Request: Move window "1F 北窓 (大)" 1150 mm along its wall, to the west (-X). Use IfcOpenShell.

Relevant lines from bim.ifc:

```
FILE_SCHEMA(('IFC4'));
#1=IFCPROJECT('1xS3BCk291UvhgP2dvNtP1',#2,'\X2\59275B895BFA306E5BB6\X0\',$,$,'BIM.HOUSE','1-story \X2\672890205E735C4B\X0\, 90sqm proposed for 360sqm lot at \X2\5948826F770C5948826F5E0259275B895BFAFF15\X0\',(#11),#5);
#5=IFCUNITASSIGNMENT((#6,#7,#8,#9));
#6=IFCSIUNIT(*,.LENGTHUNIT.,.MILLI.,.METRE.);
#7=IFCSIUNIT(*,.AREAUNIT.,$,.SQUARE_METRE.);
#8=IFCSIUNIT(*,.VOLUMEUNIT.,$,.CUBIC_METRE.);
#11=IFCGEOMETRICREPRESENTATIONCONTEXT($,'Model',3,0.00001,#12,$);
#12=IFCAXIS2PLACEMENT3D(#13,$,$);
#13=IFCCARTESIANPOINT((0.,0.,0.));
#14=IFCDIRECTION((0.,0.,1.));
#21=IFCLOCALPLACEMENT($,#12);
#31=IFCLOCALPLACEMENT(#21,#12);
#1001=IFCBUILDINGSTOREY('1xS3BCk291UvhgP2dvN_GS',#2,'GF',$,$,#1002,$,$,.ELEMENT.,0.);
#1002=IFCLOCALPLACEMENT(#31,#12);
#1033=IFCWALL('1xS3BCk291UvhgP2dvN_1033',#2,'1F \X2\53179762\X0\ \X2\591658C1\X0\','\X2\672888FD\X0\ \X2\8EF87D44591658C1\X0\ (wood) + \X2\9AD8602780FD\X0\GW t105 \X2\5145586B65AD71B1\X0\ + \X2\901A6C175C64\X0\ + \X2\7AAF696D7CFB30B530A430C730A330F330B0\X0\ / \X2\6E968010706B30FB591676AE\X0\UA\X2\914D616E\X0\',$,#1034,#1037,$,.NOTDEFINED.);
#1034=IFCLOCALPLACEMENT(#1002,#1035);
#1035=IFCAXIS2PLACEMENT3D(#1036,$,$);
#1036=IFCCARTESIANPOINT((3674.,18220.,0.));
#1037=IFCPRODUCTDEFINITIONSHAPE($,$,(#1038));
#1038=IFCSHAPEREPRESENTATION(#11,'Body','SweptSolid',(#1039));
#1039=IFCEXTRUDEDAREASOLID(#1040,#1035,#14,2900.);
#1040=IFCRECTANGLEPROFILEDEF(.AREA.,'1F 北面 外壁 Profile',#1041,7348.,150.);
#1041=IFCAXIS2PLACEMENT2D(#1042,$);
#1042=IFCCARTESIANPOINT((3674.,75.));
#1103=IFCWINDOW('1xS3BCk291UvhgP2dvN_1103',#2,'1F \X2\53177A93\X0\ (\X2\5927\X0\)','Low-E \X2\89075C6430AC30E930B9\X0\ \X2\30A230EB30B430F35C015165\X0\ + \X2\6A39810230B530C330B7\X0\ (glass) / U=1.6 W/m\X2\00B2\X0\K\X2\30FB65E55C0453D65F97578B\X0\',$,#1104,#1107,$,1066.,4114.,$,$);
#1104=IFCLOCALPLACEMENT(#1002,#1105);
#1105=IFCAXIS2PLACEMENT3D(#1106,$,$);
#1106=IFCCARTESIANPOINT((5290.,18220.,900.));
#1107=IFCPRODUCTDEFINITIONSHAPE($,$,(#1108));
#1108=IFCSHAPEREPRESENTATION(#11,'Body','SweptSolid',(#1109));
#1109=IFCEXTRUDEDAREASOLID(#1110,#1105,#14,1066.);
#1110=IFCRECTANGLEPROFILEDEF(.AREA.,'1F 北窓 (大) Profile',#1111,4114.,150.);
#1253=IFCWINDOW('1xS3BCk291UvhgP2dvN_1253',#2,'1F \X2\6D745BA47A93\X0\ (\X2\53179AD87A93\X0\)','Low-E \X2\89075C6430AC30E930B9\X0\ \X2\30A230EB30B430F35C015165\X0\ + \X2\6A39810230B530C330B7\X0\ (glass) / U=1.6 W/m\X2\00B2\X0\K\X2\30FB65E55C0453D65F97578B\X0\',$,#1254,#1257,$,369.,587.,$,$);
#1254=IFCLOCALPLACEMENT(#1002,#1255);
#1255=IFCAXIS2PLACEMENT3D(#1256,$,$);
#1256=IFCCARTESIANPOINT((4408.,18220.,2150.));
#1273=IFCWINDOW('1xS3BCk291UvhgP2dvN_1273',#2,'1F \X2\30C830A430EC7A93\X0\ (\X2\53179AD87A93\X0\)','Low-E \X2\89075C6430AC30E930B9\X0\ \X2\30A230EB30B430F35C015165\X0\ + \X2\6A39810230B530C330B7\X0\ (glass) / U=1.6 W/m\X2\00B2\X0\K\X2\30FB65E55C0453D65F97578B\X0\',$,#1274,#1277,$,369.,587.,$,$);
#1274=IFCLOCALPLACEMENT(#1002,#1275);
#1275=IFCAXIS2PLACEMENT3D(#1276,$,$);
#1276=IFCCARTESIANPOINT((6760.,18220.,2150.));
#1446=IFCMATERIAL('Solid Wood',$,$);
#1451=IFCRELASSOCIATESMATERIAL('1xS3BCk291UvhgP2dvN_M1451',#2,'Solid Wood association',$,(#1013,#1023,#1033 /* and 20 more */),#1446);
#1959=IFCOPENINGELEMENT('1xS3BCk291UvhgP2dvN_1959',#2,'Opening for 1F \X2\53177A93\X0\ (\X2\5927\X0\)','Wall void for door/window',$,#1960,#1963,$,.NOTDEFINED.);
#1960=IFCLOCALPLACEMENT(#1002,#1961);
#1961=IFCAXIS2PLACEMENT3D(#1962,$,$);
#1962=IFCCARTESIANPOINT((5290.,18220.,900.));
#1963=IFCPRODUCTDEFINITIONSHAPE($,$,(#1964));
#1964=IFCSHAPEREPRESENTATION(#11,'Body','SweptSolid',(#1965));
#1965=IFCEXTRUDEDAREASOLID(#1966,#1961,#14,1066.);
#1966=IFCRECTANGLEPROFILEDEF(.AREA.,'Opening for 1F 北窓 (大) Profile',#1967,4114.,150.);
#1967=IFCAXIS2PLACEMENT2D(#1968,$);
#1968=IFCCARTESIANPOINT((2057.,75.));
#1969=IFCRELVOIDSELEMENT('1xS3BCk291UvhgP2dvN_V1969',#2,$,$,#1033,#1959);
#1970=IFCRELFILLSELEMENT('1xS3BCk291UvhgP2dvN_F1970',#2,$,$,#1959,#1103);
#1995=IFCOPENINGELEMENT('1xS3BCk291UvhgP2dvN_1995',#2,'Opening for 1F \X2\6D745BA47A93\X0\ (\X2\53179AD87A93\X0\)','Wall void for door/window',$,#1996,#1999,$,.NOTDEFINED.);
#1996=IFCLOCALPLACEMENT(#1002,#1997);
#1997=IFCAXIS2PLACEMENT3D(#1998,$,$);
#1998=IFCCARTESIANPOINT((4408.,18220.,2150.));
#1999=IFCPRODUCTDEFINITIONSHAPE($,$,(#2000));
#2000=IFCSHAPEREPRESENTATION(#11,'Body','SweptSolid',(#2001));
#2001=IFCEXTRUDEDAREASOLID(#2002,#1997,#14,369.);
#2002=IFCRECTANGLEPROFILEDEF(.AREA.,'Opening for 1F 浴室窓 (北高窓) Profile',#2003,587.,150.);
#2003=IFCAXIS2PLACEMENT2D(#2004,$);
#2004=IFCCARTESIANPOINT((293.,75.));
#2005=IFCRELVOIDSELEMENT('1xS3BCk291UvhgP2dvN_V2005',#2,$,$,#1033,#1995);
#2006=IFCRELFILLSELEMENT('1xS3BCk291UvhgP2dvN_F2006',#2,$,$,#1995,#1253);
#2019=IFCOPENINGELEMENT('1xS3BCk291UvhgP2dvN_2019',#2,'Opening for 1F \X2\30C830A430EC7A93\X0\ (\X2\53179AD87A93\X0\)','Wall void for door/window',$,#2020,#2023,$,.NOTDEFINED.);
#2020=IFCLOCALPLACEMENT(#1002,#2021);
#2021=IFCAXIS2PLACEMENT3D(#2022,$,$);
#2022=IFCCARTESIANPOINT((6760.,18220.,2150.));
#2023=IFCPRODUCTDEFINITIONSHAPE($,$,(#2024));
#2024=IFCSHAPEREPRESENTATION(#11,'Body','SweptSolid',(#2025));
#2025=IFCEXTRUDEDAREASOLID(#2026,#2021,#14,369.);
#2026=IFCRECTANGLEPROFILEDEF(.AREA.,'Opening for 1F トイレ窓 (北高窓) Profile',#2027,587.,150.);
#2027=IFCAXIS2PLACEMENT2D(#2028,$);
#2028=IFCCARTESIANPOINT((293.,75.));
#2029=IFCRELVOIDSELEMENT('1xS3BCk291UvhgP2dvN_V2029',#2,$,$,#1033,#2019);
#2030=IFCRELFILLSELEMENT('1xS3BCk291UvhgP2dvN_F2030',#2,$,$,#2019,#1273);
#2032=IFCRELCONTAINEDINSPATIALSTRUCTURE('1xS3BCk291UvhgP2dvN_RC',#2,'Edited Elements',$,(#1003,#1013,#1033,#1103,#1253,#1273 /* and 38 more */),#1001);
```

```python
import ifcopenshell
import ifcopenshell.api.geometry
import ifcopenshell.util.placement
import ifcopenshell.util.unit

model = ifcopenshell.open("bim.ifc")
unit_scale = ifcopenshell.util.unit.calculate_unit_scale(model)

window = model.by_guid("1xS3BCk291UvhgP2dvN_1103")
opening = window.FillsVoids[0].RelatingOpeningElement
wall = opening.VoidsElements[0].RelatingBuildingElement

wall_matrix = ifcopenshell.util.placement.get_local_placement(wall.ObjectPlacement)
shift = wall_matrix[:3, 0] * -1.15 / unit_scale
before = ifcopenshell.util.placement.get_local_placement(window.ObjectPlacement)[:3, 3].copy()

# The window is not placed relative to its opening, so move both.
for product in (opening, window):
    matrix = ifcopenshell.util.placement.get_local_placement(product.ObjectPlacement)
    matrix[:3, 3] += shift
    ifcopenshell.api.geometry.edit_object_placement(model, product=product, matrix=matrix, is_si=False)

after = ifcopenshell.util.placement.get_local_placement(window.ObjectPlacement)[:3, 3]
print("window moved by", (after - before).round(3) + 0.0)

model.write("bim_updated.ifc")
```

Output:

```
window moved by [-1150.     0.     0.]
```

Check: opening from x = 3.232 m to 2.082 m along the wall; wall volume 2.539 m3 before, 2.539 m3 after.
